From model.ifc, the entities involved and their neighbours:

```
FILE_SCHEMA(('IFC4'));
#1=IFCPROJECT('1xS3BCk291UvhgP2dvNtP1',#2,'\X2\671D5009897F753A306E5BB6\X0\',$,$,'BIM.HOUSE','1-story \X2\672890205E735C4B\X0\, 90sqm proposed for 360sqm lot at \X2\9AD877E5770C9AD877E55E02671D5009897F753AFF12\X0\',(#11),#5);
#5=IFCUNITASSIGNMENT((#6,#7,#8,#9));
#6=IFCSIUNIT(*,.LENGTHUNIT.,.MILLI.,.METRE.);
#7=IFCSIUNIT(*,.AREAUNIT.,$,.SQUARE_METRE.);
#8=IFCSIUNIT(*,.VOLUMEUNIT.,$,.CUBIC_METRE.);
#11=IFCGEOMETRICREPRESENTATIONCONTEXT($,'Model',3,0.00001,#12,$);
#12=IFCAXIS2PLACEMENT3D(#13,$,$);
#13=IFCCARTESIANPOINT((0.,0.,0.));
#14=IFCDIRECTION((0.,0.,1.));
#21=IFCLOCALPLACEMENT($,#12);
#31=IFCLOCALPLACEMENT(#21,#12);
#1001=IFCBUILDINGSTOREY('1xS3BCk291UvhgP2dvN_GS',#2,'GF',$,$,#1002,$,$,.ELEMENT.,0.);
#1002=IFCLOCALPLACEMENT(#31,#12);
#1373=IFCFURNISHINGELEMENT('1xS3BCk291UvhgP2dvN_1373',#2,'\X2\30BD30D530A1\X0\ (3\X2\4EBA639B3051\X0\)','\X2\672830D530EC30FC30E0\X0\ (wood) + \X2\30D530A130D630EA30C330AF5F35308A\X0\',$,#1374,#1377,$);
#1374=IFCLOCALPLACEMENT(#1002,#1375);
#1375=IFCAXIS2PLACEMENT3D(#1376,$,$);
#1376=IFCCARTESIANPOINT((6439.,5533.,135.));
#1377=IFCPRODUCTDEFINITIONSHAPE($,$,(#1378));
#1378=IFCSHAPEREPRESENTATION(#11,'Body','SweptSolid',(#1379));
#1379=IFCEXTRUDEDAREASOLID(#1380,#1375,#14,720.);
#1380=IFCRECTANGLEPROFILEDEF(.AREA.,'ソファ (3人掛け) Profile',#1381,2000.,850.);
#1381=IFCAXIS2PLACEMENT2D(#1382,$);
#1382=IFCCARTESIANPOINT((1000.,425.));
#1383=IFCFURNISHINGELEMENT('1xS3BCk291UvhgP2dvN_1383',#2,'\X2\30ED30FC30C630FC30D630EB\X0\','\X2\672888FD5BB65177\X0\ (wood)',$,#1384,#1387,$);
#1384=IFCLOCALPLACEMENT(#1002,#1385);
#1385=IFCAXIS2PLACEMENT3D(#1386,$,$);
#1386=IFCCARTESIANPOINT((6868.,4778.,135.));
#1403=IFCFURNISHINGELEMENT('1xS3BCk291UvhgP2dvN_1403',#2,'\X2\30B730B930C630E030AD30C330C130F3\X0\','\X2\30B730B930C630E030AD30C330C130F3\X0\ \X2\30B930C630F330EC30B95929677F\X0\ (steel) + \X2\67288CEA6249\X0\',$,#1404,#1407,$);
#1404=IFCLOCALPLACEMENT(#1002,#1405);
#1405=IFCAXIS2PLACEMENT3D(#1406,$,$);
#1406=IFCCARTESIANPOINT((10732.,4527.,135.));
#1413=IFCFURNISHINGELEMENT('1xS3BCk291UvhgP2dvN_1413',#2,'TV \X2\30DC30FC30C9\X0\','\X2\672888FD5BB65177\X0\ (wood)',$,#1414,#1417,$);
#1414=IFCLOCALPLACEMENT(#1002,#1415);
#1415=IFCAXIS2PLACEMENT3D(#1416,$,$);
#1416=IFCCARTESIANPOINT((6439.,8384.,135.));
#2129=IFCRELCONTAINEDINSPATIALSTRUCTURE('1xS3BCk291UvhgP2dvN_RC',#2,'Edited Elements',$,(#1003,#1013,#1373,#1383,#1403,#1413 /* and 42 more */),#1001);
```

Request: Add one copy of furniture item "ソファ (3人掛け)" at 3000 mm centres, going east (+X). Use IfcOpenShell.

```python
import numpy as np
import ifcopenshell
import ifcopenshell.api.geometry
import ifcopenshell.api.root
import ifcopenshell.util.element
import ifcopenshell.util.placement
import ifcopenshell.util.unit

model = ifcopenshell.open("model.ifc")
unit_scale = ifcopenshell.util.unit.calculate_unit_scale(model)


def reuse_history(source, copy):
    """copy_class also copies each property set's owner history, people and application; keep the originals."""
    for rel in copy.IsDefinedBy:
        if rel.is_a("IfcRelDefinesByProperties") and (history := rel.RelatingPropertyDefinition.OwnerHistory):
            rel.RelatingPropertyDefinition.OwnerHistory = source.OwnerHistory
            ifcopenshell.util.element.remove_deep2(model, history)


source = model.by_guid("1xS3BCk291UvhgP2dvN_1373")
base = ifcopenshell.util.placement.get_local_placement(source.ObjectPlacement)
step = np.array([1.0, 0.0, 0.0]) * 3 / unit_scale

for i in range(1, 2):
    copy = ifcopenshell.api.root.copy_class(model, product=source)
    copy.Representation = ifcopenshell.util.element.copy_deep(
        model, source.Representation, exclude=["IfcGeometricRepresentationContext", "IfcRepresentationMap"]
    )
    reuse_history(source, copy)
    matrix = base.copy()
    matrix[:3, 3] += i * step
    print("added at", matrix[:3, 3].round(3) + 0.0)
    ifcopenshell.api.geometry.edit_object_placement(model, product=copy, matrix=matrix, is_si=False)

model.write("model-out.ifc")
```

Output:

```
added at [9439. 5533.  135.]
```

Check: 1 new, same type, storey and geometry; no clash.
